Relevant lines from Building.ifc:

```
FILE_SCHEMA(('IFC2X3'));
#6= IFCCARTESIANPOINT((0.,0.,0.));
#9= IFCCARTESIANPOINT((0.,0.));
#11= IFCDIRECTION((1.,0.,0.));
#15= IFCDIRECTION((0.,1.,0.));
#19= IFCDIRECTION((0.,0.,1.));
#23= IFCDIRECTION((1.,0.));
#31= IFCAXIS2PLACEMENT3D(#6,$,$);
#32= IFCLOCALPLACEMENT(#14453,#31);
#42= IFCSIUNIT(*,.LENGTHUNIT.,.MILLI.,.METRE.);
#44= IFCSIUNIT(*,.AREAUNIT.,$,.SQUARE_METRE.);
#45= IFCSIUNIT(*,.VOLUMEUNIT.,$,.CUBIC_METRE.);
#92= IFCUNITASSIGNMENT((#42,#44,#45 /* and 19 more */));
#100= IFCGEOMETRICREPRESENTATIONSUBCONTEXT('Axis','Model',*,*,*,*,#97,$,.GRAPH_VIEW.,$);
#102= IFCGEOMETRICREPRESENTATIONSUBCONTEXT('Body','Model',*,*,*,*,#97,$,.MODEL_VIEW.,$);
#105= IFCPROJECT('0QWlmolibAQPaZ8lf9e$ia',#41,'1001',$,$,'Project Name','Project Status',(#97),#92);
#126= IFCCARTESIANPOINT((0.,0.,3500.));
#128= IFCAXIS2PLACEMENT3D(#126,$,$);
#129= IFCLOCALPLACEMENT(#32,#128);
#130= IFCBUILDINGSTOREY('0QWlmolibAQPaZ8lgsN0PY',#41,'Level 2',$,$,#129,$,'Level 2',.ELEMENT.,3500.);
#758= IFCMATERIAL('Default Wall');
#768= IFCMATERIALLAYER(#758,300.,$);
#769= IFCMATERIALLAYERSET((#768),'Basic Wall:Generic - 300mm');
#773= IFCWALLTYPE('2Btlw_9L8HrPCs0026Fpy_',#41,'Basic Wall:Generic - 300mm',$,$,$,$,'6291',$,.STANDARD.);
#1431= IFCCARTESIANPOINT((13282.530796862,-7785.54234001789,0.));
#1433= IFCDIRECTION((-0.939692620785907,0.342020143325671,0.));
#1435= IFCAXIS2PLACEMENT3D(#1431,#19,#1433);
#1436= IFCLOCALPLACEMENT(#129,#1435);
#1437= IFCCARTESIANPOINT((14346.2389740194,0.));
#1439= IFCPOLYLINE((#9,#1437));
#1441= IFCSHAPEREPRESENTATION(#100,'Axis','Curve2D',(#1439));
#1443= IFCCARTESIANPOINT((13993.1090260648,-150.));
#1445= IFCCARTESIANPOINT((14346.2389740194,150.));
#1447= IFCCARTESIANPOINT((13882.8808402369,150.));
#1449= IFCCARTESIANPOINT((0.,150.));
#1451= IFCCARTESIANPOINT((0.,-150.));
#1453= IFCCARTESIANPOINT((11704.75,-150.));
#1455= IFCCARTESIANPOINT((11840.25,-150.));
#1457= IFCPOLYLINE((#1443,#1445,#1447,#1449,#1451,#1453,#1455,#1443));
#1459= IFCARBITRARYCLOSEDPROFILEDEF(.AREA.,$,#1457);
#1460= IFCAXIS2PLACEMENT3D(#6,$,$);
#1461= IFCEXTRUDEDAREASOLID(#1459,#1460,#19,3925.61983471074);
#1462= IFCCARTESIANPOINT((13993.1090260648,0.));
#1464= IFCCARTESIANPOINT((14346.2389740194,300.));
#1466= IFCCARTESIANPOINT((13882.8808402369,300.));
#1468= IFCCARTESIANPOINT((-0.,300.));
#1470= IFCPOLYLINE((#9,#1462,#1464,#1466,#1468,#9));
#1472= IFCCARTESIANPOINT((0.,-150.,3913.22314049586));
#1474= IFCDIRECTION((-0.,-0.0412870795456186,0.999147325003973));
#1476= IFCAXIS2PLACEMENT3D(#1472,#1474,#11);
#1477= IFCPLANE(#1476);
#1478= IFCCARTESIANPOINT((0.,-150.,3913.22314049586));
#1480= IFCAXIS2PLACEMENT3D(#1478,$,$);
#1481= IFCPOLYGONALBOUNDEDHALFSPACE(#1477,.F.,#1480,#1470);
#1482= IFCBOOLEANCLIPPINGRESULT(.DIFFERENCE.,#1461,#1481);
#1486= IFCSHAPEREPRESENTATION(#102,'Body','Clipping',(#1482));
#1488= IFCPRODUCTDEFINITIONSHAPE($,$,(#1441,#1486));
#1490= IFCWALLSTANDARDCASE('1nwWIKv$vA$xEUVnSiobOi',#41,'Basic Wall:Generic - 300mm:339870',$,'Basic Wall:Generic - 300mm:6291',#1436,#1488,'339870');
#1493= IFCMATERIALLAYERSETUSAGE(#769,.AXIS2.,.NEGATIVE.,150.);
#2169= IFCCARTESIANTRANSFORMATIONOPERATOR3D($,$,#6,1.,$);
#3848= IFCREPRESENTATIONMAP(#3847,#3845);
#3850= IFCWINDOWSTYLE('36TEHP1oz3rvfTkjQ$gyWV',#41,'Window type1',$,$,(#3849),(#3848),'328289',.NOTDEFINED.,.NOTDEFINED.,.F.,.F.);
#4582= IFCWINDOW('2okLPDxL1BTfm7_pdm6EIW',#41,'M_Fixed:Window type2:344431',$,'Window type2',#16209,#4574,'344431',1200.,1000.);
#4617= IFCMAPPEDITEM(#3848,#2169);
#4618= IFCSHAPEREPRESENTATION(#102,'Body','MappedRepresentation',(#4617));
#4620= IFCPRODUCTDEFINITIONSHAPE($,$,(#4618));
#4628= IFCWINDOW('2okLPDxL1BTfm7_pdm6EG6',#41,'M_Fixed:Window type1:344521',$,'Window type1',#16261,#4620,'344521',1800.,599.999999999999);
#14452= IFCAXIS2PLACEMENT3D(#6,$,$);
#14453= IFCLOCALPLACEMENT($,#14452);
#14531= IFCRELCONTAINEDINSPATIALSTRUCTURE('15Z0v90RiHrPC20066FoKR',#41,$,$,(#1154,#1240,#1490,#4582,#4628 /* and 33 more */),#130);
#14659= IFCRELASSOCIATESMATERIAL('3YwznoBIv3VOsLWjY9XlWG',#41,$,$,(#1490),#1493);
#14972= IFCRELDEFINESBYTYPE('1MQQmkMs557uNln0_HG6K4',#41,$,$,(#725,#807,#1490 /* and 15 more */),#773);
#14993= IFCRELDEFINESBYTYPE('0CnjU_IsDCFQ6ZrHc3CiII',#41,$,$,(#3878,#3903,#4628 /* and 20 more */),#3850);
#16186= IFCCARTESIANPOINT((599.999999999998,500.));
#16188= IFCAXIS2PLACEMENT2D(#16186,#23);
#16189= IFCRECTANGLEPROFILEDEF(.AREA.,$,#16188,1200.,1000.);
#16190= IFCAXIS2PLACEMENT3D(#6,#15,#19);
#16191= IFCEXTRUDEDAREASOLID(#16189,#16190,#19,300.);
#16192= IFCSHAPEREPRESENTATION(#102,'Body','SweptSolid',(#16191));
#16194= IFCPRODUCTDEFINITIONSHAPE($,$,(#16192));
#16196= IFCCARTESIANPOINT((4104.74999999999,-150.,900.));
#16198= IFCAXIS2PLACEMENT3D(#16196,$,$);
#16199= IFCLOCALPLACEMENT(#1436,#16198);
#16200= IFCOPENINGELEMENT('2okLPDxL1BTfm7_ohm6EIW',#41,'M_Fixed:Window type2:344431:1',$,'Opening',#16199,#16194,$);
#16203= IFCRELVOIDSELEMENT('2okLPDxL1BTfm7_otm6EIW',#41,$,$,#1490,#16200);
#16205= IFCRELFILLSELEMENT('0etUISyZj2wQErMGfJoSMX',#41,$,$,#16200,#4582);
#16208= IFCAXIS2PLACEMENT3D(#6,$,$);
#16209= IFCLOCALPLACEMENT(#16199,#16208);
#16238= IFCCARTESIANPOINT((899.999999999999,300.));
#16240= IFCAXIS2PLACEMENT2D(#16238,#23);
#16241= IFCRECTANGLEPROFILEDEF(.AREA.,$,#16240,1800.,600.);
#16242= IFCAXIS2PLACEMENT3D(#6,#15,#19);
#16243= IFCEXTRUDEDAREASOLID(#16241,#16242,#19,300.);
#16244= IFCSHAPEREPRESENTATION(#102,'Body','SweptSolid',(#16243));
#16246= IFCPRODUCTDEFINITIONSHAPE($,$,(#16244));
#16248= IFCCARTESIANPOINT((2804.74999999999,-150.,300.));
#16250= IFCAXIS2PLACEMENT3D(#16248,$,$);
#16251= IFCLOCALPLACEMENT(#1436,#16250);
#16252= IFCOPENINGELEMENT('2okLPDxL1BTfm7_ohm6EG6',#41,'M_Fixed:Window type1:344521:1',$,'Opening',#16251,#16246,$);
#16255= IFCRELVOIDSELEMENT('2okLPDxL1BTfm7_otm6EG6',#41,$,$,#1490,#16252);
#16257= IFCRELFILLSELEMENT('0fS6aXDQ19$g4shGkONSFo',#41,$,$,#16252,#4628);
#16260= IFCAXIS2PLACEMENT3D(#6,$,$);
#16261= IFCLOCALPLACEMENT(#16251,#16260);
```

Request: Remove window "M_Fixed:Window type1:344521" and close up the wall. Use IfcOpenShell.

```python
import ifcopenshell
import ifcopenshell.api.feature
import ifcopenshell.api.root
import ifcopenshell.geom
import ifcopenshell.util.shape

model = ifcopenshell.open("Building.ifc")
settings = ifcopenshell.geom.settings()


def volume(element):
    """Net volume in cubic metres, openings subtracted."""
    shape = ifcopenshell.geom.create_shape(settings, element)
    return ifcopenshell.util.shape.get_volume(shape.geometry)


window = model.by_id(4628)
opening = window.FillsVoids[0].RelatingOpeningElement
wall = opening.VoidsElements[0].RelatingBuildingElement
before = volume(wall)

ifcopenshell.api.root.remove_product(model, product=window)
ifcopenshell.api.feature.remove_feature(model, feature=opening)

after = volume(wall)

print(f"wall volume {before:.3f} -> {after:.3f} m3")

model.write("Building-out.ifc")
```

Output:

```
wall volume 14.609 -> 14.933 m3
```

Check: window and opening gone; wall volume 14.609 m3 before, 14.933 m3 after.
